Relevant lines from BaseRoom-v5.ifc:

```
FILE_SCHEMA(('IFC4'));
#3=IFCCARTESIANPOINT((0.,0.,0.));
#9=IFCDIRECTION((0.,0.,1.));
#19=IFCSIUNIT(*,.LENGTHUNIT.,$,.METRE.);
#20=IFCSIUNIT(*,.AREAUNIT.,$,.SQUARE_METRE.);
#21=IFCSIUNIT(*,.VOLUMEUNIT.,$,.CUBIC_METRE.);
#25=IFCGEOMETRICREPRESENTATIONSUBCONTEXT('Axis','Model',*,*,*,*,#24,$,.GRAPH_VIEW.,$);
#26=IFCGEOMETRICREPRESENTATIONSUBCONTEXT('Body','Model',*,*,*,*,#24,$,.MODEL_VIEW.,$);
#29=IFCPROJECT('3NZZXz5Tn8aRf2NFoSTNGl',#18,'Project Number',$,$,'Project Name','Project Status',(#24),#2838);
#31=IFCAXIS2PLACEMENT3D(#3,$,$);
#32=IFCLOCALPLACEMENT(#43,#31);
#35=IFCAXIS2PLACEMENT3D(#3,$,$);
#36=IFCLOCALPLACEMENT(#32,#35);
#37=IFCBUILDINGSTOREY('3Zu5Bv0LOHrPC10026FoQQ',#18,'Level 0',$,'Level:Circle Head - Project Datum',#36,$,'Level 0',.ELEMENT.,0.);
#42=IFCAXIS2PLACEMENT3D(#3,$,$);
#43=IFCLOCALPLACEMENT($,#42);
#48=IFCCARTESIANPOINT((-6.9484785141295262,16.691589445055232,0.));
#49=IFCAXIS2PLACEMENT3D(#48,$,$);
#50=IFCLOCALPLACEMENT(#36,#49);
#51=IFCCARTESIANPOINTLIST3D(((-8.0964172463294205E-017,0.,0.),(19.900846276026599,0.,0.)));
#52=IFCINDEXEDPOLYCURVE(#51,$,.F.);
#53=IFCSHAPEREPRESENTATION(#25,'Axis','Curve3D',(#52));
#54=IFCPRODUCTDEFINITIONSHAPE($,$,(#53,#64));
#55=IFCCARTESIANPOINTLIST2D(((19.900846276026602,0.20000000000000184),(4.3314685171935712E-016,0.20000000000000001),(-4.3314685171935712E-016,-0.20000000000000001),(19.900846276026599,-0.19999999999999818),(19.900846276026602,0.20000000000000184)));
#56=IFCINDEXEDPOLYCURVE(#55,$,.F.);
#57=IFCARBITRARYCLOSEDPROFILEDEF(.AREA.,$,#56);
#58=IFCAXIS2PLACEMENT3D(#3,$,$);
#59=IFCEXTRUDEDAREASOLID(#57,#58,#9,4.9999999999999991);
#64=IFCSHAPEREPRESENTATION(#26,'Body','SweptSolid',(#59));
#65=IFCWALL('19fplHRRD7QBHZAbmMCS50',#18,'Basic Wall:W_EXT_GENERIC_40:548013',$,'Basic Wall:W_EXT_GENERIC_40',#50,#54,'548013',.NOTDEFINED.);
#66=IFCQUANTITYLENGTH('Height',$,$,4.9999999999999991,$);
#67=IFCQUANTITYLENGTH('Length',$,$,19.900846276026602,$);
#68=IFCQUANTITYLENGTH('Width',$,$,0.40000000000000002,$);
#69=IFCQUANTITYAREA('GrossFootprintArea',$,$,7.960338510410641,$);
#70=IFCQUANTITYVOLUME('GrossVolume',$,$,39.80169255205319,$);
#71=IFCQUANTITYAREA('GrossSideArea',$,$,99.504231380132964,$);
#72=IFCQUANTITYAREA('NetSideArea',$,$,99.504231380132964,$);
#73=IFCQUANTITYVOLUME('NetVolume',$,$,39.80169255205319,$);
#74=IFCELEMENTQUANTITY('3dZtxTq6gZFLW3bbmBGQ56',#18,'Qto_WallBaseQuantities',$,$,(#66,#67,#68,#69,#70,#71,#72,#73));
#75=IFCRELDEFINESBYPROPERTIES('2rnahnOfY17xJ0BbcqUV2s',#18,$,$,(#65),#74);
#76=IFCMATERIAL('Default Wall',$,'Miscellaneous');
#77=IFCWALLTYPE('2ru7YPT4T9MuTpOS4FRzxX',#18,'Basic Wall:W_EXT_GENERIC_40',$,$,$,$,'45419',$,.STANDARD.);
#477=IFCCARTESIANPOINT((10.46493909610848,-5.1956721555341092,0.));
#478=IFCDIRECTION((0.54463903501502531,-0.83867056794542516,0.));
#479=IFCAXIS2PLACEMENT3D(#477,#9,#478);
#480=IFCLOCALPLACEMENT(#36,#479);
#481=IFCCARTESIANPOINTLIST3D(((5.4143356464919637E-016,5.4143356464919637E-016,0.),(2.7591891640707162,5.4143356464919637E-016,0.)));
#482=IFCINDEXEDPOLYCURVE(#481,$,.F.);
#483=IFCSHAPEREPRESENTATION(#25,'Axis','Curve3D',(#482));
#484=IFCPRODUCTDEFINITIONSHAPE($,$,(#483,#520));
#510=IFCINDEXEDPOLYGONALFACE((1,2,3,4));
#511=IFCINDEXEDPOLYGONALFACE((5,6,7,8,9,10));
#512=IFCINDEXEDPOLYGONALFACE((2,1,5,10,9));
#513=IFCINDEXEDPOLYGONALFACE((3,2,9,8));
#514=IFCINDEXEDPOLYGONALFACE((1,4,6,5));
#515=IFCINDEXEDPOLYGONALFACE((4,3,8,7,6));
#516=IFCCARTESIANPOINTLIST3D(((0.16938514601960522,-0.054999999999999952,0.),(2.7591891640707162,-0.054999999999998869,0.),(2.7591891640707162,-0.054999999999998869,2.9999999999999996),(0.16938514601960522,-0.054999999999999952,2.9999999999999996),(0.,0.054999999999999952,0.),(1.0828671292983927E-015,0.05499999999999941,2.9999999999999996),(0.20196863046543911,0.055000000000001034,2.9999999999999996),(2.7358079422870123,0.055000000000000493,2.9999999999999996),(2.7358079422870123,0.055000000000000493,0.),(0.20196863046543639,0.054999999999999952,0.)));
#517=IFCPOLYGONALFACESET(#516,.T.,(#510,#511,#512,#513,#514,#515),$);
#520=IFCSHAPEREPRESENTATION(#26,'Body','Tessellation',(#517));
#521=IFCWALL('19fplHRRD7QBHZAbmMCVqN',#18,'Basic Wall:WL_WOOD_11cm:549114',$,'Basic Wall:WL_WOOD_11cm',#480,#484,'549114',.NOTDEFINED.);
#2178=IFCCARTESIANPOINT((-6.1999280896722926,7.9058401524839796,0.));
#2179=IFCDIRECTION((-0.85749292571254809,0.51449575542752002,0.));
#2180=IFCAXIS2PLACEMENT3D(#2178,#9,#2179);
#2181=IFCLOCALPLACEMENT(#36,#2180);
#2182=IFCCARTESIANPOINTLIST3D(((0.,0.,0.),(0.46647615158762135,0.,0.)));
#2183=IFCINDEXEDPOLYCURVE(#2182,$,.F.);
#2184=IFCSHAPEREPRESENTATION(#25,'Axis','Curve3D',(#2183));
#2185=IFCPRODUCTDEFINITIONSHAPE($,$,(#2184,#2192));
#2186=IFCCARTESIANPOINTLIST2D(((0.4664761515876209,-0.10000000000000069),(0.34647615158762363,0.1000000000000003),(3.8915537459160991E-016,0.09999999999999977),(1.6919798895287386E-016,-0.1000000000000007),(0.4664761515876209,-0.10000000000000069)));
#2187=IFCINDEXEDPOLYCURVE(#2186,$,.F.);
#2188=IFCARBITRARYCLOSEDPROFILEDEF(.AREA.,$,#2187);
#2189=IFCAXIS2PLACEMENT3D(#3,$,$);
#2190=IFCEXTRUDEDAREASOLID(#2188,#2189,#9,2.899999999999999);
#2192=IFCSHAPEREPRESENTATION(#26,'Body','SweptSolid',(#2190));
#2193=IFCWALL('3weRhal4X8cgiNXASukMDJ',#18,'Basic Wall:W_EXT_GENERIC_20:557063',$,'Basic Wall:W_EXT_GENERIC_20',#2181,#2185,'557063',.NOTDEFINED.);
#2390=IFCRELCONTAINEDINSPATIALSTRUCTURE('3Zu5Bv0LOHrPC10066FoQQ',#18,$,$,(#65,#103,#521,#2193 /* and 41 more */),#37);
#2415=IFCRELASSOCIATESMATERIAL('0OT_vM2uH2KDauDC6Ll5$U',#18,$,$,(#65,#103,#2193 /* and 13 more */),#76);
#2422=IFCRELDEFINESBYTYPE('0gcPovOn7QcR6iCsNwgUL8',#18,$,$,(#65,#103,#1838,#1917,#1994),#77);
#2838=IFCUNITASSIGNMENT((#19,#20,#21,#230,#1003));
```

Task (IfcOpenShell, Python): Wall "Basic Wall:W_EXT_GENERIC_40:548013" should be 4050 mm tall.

```python
import ifcopenshell
import ifcopenshell.api.pset
import ifcopenshell.geom
import ifcopenshell.util.element
import ifcopenshell.util.representation
import ifcopenshell.util.shape
import ifcopenshell.util.unit

model = ifcopenshell.open("BaseRoom-v5.ifc")
unit_scale = ifcopenshell.util.unit.calculate_unit_scale(model)
area_scale = ifcopenshell.util.unit.calculate_unit_scale(model, "AREAUNIT")
volume_scale = ifcopenshell.util.unit.calculate_unit_scale(model, "VOLUMEUNIT")
settings = ifcopenshell.geom.settings()


def volume(element):
    """Net volume in cubic metres, openings subtracted."""
    shape = ifcopenshell.geom.create_shape(settings, element)
    return ifcopenshell.util.shape.get_volume(shape.geometry)


wall = model.by_guid("19fplHRRD7QBHZAbmMCS50")
before = volume(wall)

body = ifcopenshell.util.representation.get_representation(wall, "Model", "Body")
solid = body.Items[0]
old_height = solid.Depth
solid.Depth = 4.05 / unit_scale
after = volume(wall)
thickness = 0.4  # wall thickness in metres

# Update the stored height, areas and volumes.
qto = model.by_id(ifcopenshell.util.element.get_pset(wall, "Qto_WallBaseQuantities", should_inherit=False)["id"])
ifcopenshell.api.pset.edit_qto(model, qto=qto, properties={
    "Height": solid.Depth,
    "GrossVolume": ifcopenshell.util.element.get_pset(wall, "Qto_WallBaseQuantities", "GrossVolume") * solid.Depth / old_height,
    "GrossSideArea": ifcopenshell.util.element.get_pset(wall, "Qto_WallBaseQuantities", "GrossSideArea") * solid.Depth / old_height,
    "NetSideArea": after / thickness / area_scale,
    "NetVolume": after / volume_scale,
})

print(f"height {old_height:g} -> {solid.Depth:g}, volume {before:.3f} -> {after:.3f} m3")

model.write("BaseRoom-v5_rev.ifc")
```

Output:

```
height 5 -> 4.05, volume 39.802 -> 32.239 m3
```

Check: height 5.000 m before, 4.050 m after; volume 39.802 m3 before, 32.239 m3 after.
